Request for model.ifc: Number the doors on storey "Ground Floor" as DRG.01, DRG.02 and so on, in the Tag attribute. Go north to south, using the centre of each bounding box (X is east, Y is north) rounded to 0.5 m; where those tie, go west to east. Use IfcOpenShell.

First a look at what the model holds.

```python
import ifcopenshell
import ifcopenshell.util.element
import ifcopenshell.util.placement

model = ifcopenshell.open("model.ifc")
print(model.schema)
storey = next(s for s in model.by_type("IfcBuildingStorey") if s.Name == "Ground Floor")
doors = [e for e in ifcopenshell.util.element.get_decomposition(storey) if e.is_a("IfcDoor")]
for e in sorted(doors, key=lambda e: e.id()):
    origin = ifcopenshell.util.placement.get_local_placement(e.ObjectPlacement)[:3, 3]
    print(e.id(), e.Tag, e.Name, origin.round(2) + 0.0, sep=" | ")
```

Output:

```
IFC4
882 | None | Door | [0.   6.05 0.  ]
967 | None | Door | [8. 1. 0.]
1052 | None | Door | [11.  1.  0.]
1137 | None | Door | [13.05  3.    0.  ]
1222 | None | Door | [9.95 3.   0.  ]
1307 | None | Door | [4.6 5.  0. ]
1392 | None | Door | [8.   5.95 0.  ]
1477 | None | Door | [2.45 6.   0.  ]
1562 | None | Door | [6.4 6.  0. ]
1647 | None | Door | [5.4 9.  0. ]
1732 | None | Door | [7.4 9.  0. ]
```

```python
import ifcopenshell
import ifcopenshell.geom
import ifcopenshell.util.element
import ifcopenshell.util.shape

model = ifcopenshell.open("model.ifc")
settings = ifcopenshell.geom.settings()
settings.set("use-world-coords", True)


def centre(element):
    shape = ifcopenshell.geom.create_shape(settings, element)
    return ifcopenshell.util.shape.get_bbox_centroid(shape.geometry)


storey = next(s for s in model.by_type("IfcBuildingStorey") if s.Name == "Ground Floor")
doors = [e for e in ifcopenshell.util.element.get_decomposition(storey) if e.is_a("IfcDoor")]

# Insertion points can sit at a corner or the storey origin, so sort by the geometry (in metres).
centres = {e: centre(e) for e in doors}
doors.sort(key=lambda e: (-round(centres[e][1] / 0.5), centres[e][0]))

for i, e in enumerate(doors, start=1):
    number = f"DRG.{i:02d}"
    e.Tag = number
    print(e.id(), number)

model.write("model_edited.ifc")
```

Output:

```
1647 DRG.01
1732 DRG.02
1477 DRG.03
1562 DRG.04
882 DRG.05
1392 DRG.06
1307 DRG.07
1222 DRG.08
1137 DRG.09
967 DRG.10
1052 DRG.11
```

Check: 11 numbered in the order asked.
